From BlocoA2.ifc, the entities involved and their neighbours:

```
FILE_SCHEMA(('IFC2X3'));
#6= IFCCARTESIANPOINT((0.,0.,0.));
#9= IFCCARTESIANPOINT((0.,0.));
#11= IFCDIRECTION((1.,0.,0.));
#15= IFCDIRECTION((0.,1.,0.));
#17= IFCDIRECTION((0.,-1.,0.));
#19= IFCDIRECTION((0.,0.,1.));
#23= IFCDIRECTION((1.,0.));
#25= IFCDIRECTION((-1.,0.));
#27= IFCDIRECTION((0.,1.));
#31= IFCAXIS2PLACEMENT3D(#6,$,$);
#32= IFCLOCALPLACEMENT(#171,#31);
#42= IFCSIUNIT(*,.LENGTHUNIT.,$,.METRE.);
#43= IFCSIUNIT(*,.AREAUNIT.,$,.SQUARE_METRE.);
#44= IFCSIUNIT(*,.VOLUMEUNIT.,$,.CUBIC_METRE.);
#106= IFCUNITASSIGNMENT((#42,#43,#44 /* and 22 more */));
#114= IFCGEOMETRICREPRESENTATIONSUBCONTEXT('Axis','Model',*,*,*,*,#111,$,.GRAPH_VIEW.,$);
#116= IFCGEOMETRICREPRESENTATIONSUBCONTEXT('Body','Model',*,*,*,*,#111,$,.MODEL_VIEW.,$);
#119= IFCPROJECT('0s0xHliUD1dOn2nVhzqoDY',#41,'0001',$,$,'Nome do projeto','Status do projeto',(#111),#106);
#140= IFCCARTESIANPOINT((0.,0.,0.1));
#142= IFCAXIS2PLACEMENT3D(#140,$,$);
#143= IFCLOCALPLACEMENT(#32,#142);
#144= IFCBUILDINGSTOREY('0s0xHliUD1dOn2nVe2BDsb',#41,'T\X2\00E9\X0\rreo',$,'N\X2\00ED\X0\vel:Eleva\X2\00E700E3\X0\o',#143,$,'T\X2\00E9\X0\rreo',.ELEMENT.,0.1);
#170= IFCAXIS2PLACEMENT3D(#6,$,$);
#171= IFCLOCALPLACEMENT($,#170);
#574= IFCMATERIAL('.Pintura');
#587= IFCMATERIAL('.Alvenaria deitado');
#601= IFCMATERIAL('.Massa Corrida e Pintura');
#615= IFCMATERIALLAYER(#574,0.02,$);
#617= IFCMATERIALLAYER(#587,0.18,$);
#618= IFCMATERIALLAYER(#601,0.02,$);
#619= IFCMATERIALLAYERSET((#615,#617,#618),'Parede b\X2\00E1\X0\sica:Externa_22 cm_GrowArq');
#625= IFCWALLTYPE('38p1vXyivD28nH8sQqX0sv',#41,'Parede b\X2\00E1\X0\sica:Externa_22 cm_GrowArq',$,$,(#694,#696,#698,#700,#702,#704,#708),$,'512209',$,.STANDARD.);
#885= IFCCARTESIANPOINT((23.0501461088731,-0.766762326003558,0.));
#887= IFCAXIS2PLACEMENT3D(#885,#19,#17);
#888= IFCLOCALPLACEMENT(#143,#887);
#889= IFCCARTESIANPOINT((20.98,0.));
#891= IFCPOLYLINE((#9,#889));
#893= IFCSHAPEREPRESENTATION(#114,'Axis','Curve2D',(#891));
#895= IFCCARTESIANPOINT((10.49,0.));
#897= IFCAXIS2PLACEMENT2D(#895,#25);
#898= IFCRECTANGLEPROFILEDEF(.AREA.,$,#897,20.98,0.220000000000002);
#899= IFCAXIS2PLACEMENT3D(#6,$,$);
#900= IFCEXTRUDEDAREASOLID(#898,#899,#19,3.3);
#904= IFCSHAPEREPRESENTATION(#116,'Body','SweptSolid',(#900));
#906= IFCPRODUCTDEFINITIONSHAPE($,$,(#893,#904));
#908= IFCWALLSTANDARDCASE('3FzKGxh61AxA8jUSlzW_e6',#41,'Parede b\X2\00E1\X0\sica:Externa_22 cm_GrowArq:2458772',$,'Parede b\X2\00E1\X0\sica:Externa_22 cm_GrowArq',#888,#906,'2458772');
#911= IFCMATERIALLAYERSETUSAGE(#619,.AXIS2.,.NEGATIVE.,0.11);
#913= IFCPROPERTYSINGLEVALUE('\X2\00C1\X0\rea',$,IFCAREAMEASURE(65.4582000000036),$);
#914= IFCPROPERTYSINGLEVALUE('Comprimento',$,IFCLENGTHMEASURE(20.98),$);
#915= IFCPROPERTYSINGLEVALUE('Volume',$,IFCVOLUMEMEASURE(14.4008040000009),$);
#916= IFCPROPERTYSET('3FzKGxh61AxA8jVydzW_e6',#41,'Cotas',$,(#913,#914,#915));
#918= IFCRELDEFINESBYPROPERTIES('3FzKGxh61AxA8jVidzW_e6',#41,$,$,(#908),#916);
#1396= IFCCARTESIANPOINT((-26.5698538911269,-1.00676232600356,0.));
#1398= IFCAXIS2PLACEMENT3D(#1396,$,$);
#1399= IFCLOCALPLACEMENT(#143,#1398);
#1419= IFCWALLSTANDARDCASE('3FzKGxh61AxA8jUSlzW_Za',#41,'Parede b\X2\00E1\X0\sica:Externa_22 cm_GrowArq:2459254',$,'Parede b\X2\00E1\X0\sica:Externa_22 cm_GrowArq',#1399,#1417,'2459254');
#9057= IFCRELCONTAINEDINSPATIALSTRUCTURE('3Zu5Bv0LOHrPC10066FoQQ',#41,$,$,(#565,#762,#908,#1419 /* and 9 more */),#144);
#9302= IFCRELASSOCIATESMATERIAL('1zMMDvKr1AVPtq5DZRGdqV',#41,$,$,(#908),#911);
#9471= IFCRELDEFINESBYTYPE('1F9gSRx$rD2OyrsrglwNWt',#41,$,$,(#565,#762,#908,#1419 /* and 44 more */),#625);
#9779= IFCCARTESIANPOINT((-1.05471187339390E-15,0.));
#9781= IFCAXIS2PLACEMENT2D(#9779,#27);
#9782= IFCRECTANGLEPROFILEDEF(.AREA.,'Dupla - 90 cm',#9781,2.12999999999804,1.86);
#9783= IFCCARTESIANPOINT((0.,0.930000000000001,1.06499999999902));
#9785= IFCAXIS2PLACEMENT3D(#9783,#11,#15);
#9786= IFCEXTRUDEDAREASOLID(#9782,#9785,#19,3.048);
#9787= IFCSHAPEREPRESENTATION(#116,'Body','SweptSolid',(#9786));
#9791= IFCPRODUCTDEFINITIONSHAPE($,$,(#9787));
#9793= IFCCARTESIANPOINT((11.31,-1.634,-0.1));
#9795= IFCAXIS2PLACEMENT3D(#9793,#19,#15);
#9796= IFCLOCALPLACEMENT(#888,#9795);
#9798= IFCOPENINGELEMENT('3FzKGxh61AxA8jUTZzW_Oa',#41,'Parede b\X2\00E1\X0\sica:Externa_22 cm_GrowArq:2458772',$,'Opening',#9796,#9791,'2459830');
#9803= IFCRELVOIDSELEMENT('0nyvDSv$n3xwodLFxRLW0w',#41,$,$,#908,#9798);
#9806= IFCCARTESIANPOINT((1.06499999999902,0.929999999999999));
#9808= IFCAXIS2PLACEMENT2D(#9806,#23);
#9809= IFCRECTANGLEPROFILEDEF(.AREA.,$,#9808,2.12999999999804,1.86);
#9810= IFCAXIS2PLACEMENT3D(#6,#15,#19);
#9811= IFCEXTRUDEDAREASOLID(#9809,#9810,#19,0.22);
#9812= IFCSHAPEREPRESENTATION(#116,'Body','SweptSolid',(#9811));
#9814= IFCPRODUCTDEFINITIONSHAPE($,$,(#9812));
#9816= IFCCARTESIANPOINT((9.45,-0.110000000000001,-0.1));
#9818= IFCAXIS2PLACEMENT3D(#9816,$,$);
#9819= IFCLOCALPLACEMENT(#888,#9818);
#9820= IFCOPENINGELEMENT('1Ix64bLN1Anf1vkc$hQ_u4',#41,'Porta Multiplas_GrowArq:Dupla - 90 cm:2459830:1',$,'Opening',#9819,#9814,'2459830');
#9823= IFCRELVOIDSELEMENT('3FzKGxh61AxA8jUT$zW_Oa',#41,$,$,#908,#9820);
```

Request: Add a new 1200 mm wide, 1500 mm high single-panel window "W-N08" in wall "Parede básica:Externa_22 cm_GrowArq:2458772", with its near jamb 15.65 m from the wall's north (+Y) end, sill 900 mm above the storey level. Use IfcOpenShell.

```python
import numpy as np
import ifcopenshell
import ifcopenshell.api.feature
import ifcopenshell.api.geometry
import ifcopenshell.api.pset
import ifcopenshell.api.root
import ifcopenshell.api.spatial
import ifcopenshell.api.type
import ifcopenshell.geom
import ifcopenshell.util.element
import ifcopenshell.util.placement
import ifcopenshell.util.representation
import ifcopenshell.util.shape
import ifcopenshell.util.unit

model = ifcopenshell.open("BlocoA2.ifc")
unit_scale = ifcopenshell.util.unit.calculate_unit_scale(model)
area_scale = ifcopenshell.util.unit.calculate_unit_scale(model, "AREAUNIT")
volume_scale = ifcopenshell.util.unit.calculate_unit_scale(model, "VOLUMEUNIT")
settings = ifcopenshell.geom.settings()


def volume(element):
    """Net volume in cubic metres, openings subtracted."""
    shape = ifcopenshell.geom.create_shape(settings, element)
    return ifcopenshell.util.shape.get_volume(shape.geometry)


wall = model.by_guid("3FzKGxh61AxA8jUSlzW_e6")
storey = ifcopenshell.util.element.get_container(wall, ifc_class="IfcBuildingStorey")
context = ifcopenshell.util.representation.get_context(model, "Model", "Body", "MODEL_VIEW")
before = volume(wall)

width, height, from_end, sill = 1.2, 1.5, 15.65, 0.9  # metres

# The wall runs along its own X axis, and the end named is its -X end.
wall_shape = ifcopenshell.geom.create_shape(settings, wall)
x, y, z = ifcopenshell.util.shape.get_vertices(wall_shape.geometry).T
start = x.min() + from_end
face, thickness = float(y.min()), float(y.max() - y.min())
wall_matrix = ifcopenshell.util.placement.get_local_placement(wall.ObjectPlacement)
level = ifcopenshell.util.placement.get_local_placement(storey.ObjectPlacement)[2, 3]


def in_wall(x, y):
    """Placement at x, y metres in the wall's axes, at sill height."""
    matrix = wall_matrix.copy()
    matrix[:, 3] = wall_matrix @ np.array([x / unit_scale, y / unit_scale, 0.0, 1.0])
    matrix[2, 3] = level + sill / unit_scale
    return matrix


# Opening: a box that overshoots both wall faces by 50 mm.
opening = ifcopenshell.api.root.create_entity(model, ifc_class="IfcOpeningElement")
box = ifcopenshell.api.geometry.add_wall_representation(
    model, context=context, length=width, height=height, thickness=thickness + 0.1
)
ifcopenshell.api.geometry.assign_representation(model, product=opening, representation=box)
ifcopenshell.api.geometry.edit_object_placement(model, product=opening, matrix=in_wall(start, face - 0.05), is_si=False)
ifcopenshell.api.feature.add_feature(model, feature=opening, element=wall)

window = ifcopenshell.api.root.create_entity(model, ifc_class="IfcWindow", name="W-N08")
window.OverallWidth, window.OverallHeight = width / unit_scale, height / unit_scale
body = ifcopenshell.api.geometry.add_window_representation(
    model,
    context=context,
    overall_width=window.OverallWidth,
    overall_height=window.OverallHeight,
    partition_type="SINGLE_PANEL",
)
ifcopenshell.api.geometry.assign_representation(model, product=window, representation=body)
ifcopenshell.api.spatial.assign_container(model, products=[window], relating_structure=storey)
fills = ifcopenshell.api.feature.add_filling(model, opening=opening, element=window)
fills.OwnerHistory = window.OwnerHistory  # required in IFC2X3

# IFC2X3 keeps the operation on the window style.
style = ifcopenshell.api.root.create_entity(model, ifc_class="IfcWindowStyle", name="W-N08")
style.OperationType, style.ConstructionType = "SINGLE_PANEL", "NOTDEFINED"
style.ParameterTakesPrecedence = style.Sizeable = False
ifcopenshell.api.type.assign_type(model, related_objects=[window], relating_type=style)

# Centre the window in the wall's thickness.
ifcopenshell.api.geometry.edit_object_placement(model, product=window, matrix=in_wall(start, face), is_si=False)
window_shape = ifcopenshell.geom.create_shape(settings, window)
depth = ifcopenshell.util.shape.get_vertices(window_shape.geometry)[:, 1]
offset = face + thickness / 2 - (depth.min() + depth.max()) / 2
ifcopenshell.api.geometry.edit_object_placement(model, product=window, matrix=in_wall(start, offset), is_si=False)

after = volume(wall)

# Update the wall's stored quantities.
pset = model.by_id(ifcopenshell.util.element.get_pset(wall, "Cotas", should_inherit=False)["id"])
ifcopenshell.api.pset.edit_pset(model, pset=pset, properties={
    "Área": model.create_entity("IfcAreaMeasure", after / thickness / area_scale),
    "Volume": model.create_entity("IfcVolumeMeasure", after / volume_scale),
})

print(f"wall volume {before:.3f} -> {after:.3f} m3")

model.write("BlocoA2_rev.ifc")
```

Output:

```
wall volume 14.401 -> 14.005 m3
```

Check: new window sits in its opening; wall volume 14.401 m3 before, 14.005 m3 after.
